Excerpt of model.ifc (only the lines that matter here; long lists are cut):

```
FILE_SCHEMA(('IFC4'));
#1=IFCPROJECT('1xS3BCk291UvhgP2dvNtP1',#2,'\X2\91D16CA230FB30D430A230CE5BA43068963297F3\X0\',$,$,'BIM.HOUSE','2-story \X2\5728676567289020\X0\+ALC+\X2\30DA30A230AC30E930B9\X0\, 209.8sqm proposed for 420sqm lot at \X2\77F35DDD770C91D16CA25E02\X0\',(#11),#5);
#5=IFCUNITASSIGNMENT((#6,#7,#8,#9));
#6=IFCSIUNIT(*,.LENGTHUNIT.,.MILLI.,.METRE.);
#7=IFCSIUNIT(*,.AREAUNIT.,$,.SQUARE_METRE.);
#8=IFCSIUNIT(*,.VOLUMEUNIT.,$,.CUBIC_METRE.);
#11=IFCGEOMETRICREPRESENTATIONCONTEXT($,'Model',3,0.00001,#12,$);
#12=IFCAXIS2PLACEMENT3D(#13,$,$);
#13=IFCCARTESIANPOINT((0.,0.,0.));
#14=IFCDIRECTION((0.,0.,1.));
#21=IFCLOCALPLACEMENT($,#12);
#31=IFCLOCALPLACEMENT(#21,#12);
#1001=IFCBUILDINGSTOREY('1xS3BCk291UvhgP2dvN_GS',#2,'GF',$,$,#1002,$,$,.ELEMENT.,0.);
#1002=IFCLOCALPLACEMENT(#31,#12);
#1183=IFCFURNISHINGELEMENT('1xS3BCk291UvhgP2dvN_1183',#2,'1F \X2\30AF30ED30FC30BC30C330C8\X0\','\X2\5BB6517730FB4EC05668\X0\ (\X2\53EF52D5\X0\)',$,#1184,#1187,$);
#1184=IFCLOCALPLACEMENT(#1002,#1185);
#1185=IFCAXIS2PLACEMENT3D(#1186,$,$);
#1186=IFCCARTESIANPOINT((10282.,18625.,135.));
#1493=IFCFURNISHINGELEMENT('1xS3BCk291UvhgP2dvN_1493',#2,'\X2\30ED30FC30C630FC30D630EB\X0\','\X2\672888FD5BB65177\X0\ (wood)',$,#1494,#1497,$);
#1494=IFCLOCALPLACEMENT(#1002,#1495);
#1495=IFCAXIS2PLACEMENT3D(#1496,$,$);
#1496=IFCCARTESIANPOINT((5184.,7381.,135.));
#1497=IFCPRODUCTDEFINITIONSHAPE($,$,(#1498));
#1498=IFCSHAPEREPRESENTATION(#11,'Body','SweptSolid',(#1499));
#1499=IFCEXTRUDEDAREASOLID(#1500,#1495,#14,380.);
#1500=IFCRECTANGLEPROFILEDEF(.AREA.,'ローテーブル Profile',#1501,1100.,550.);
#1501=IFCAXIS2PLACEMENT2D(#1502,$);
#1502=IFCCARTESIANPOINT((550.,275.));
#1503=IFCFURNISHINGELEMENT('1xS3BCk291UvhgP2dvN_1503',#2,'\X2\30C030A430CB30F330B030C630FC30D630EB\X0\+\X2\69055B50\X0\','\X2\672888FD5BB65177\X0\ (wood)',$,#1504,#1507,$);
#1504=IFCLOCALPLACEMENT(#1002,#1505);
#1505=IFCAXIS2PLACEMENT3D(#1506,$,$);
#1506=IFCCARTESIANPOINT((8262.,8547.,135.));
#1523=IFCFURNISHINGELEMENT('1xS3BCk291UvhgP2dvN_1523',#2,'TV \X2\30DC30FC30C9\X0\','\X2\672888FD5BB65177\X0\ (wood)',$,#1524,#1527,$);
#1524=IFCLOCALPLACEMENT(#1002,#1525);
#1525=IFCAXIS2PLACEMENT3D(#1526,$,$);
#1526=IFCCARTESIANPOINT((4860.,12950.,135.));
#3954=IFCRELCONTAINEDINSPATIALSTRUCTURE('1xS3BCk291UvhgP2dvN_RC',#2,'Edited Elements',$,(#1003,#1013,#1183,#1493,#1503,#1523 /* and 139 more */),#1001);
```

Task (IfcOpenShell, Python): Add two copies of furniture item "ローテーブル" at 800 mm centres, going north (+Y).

```python
import numpy as np
import ifcopenshell
import ifcopenshell.api.geometry
import ifcopenshell.api.root
import ifcopenshell.util.element
import ifcopenshell.util.placement
import ifcopenshell.util.unit

model = ifcopenshell.open("model.ifc")
unit_scale = ifcopenshell.util.unit.calculate_unit_scale(model)


def reuse_history(source, copy):
    """copy_class also copies each property set's owner history, people and application; keep the originals."""
    for rel in copy.IsDefinedBy:
        if rel.is_a("IfcRelDefinesByProperties") and (history := rel.RelatingPropertyDefinition.OwnerHistory):
            rel.RelatingPropertyDefinition.OwnerHistory = source.OwnerHistory
            ifcopenshell.util.element.remove_deep2(model, history)


source = model.by_id(1493)
base = ifcopenshell.util.placement.get_local_placement(source.ObjectPlacement)
step = np.array([0.0, 1.0, 0.0]) * 0.8 / unit_scale

for i in range(1, 3):
    copy = ifcopenshell.api.root.copy_class(model, product=source)
    copy.Representation = ifcopenshell.util.element.copy_deep(
        model, source.Representation, exclude=["IfcGeometricRepresentationContext", "IfcRepresentationMap"]
    )
    reuse_history(source, copy)
    matrix = base.copy()
    matrix[:3, 3] += i * step
    print("added at", matrix[:3, 3].round(3) + 0.0)
    ifcopenshell.api.geometry.edit_object_placement(model, product=copy, matrix=matrix, is_si=False)

model.write("model_edited.ifc")
```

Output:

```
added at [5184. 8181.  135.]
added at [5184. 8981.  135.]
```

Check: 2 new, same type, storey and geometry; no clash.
